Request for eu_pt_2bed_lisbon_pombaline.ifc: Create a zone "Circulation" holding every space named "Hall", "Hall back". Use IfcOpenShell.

First a look at what the model holds.

```python
import ifcopenshell

model = ifcopenshell.open("eu_pt_2bed_lisbon_pombaline.ifc")
print(model.schema)
seen = {}
for space in model.by_type("IfcSpace"):
    seen[space.LongName] = seen.get(space.LongName, 0) + 1
for name, count in sorted(seen.items(), key=str):
    print(count, "x", name)
print("zones:", [z.Name for z in model.by_type("IfcZone")][:20])
```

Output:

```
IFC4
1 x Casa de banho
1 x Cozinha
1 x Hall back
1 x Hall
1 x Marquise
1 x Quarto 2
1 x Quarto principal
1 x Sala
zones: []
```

```python
import ifcopenshell
import ifcopenshell.api.group
import ifcopenshell.api.root

model = ifcopenshell.open("eu_pt_2bed_lisbon_pombaline.ifc")

names = {"Hall", "Hall back"}
spaces = [s for s in model.by_type("IfcSpace") if s.LongName in names]

zone = ifcopenshell.api.root.create_entity(model, ifc_class="IfcZone", name="Circulation")
ifcopenshell.api.group.assign_group(model, products=spaces, group=zone)
print(len(spaces), "spaces in", zone.Name)

model.write("eu_pt_2bed_lisbon_pombaline_updated.ifc")
```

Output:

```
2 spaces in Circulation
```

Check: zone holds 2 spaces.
